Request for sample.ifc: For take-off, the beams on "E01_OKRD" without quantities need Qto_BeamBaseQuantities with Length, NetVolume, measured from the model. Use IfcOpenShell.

First a look at what the model holds.

```python
import ifcopenshell
import ifcopenshell.util.element
import ifcopenshell.util.unit

model = ifcopenshell.open("sample.ifc")
print(model.schema)
for unit_type in ("LENGTHUNIT", "AREAUNIT", "VOLUMEUNIT"):
    print(unit_type, ifcopenshell.util.unit.calculate_unit_scale(model, unit_type))
storey = next(s for s in model.by_type("IfcBuildingStorey") if s.Name == "E01_OKRD")
beams = [e for e in ifcopenshell.util.element.get_decomposition(storey) if e.is_a("IfcBeam")]
for e in sorted(beams, key=lambda e: e.id()):
    print(e.id(), e.is_a(), e.Name, list(ifcopenshell.util.element.get_psets(e, qtos_only=True)), sep=" | ")
```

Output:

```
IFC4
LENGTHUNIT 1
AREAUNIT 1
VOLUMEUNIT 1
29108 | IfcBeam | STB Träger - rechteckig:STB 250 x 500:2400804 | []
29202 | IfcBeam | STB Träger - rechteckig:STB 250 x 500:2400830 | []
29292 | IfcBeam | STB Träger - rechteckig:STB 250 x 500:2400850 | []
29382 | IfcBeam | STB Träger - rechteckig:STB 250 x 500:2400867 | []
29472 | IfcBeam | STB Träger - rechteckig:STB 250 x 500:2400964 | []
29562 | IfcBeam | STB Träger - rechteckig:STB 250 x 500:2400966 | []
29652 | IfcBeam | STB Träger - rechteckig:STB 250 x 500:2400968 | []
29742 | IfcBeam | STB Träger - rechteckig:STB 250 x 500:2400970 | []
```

```python
import ifcopenshell
import ifcopenshell.api.pset
import ifcopenshell.geom
import ifcopenshell.util.element
import ifcopenshell.util.shape
import ifcopenshell.util.unit

model = ifcopenshell.open("sample.ifc")
unit_scale = ifcopenshell.util.unit.calculate_unit_scale(model)
volume_scale = ifcopenshell.util.unit.calculate_unit_scale(model, "VOLUMEUNIT")
settings = ifcopenshell.geom.settings()

storey = next(s for s in model.by_type("IfcBuildingStorey") if s.Name == "E01_OKRD")
beams = [e for e in ifcopenshell.util.element.get_decomposition(storey) if e.is_a("IfcBeam")]

for e in sorted(beams, key=lambda e: e.id()):
    if ifcopenshell.util.element.get_psets(e, qtos_only=True, should_inherit=False):
        continue
    # Geometry comes back in metres, in the element's own axes.
    shape = ifcopenshell.geom.create_shape(settings, e)
    values = {
        "Length": ifcopenshell.util.shape.get_max_xyz(shape.geometry) / unit_scale,
        "NetVolume": ifcopenshell.util.shape.get_volume(shape.geometry) / volume_scale,
    }
    qto = ifcopenshell.api.pset.add_qto(model, product=e, name="Qto_BeamBaseQuantities")
    ifcopenshell.api.pset.edit_qto(model, qto=qto, properties=values)
    print(e.id(), {k: round(v, 3) for k, v in values.items()})

model.write("sample_rev.ifc")
```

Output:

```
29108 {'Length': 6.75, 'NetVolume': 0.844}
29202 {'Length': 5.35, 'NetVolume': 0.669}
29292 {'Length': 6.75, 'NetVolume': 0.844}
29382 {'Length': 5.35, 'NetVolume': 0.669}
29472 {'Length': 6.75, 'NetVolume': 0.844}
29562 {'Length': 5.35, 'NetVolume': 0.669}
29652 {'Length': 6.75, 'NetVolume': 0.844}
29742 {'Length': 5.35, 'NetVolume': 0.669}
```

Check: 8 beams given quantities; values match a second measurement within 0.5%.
